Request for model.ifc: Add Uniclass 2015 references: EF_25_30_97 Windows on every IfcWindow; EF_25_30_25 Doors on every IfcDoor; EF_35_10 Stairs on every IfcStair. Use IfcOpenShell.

First a look at what the model holds.

```python
import ifcopenshell

model = ifcopenshell.open("model.ifc")
print(model.schema)
print("classifications:", [c.Name for c in model.by_type("IfcClassification")])
for ifc_class in ("IfcDoor", "IfcRoof", "IfcStair", "IfcWall", "IfcWindow"):
    print(ifc_class, len(model.by_type(ifc_class)))
```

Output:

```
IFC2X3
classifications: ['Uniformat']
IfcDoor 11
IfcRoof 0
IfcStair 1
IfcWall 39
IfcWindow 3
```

```python
import ifcopenshell
import ifcopenshell.api.classification

model = ifcopenshell.open("model.ifc")

# IFC2X3 requires Source and Edition and has no link from the project to the system.
system = model.create_entity("IfcClassification", Source="NBS", Edition="2015", Name="Uniclass 2015")

codes = {
    "IfcWindow": ("EF_25_30_97", "Windows"),
    "IfcDoor": ("EF_25_30_25", "Doors"),
    "IfcStair": ("EF_35_10", "Stairs"),
}
for ifc_class, (code, name) in codes.items():
    products = model.by_type(ifc_class)
    ifcopenshell.api.classification.add_reference(
        model, products=products, classification=system, identification=code, name=name
    )
    print(code, len(products))

model.write("model_rev.ifc")
```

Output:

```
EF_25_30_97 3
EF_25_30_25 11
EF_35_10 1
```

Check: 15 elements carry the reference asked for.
